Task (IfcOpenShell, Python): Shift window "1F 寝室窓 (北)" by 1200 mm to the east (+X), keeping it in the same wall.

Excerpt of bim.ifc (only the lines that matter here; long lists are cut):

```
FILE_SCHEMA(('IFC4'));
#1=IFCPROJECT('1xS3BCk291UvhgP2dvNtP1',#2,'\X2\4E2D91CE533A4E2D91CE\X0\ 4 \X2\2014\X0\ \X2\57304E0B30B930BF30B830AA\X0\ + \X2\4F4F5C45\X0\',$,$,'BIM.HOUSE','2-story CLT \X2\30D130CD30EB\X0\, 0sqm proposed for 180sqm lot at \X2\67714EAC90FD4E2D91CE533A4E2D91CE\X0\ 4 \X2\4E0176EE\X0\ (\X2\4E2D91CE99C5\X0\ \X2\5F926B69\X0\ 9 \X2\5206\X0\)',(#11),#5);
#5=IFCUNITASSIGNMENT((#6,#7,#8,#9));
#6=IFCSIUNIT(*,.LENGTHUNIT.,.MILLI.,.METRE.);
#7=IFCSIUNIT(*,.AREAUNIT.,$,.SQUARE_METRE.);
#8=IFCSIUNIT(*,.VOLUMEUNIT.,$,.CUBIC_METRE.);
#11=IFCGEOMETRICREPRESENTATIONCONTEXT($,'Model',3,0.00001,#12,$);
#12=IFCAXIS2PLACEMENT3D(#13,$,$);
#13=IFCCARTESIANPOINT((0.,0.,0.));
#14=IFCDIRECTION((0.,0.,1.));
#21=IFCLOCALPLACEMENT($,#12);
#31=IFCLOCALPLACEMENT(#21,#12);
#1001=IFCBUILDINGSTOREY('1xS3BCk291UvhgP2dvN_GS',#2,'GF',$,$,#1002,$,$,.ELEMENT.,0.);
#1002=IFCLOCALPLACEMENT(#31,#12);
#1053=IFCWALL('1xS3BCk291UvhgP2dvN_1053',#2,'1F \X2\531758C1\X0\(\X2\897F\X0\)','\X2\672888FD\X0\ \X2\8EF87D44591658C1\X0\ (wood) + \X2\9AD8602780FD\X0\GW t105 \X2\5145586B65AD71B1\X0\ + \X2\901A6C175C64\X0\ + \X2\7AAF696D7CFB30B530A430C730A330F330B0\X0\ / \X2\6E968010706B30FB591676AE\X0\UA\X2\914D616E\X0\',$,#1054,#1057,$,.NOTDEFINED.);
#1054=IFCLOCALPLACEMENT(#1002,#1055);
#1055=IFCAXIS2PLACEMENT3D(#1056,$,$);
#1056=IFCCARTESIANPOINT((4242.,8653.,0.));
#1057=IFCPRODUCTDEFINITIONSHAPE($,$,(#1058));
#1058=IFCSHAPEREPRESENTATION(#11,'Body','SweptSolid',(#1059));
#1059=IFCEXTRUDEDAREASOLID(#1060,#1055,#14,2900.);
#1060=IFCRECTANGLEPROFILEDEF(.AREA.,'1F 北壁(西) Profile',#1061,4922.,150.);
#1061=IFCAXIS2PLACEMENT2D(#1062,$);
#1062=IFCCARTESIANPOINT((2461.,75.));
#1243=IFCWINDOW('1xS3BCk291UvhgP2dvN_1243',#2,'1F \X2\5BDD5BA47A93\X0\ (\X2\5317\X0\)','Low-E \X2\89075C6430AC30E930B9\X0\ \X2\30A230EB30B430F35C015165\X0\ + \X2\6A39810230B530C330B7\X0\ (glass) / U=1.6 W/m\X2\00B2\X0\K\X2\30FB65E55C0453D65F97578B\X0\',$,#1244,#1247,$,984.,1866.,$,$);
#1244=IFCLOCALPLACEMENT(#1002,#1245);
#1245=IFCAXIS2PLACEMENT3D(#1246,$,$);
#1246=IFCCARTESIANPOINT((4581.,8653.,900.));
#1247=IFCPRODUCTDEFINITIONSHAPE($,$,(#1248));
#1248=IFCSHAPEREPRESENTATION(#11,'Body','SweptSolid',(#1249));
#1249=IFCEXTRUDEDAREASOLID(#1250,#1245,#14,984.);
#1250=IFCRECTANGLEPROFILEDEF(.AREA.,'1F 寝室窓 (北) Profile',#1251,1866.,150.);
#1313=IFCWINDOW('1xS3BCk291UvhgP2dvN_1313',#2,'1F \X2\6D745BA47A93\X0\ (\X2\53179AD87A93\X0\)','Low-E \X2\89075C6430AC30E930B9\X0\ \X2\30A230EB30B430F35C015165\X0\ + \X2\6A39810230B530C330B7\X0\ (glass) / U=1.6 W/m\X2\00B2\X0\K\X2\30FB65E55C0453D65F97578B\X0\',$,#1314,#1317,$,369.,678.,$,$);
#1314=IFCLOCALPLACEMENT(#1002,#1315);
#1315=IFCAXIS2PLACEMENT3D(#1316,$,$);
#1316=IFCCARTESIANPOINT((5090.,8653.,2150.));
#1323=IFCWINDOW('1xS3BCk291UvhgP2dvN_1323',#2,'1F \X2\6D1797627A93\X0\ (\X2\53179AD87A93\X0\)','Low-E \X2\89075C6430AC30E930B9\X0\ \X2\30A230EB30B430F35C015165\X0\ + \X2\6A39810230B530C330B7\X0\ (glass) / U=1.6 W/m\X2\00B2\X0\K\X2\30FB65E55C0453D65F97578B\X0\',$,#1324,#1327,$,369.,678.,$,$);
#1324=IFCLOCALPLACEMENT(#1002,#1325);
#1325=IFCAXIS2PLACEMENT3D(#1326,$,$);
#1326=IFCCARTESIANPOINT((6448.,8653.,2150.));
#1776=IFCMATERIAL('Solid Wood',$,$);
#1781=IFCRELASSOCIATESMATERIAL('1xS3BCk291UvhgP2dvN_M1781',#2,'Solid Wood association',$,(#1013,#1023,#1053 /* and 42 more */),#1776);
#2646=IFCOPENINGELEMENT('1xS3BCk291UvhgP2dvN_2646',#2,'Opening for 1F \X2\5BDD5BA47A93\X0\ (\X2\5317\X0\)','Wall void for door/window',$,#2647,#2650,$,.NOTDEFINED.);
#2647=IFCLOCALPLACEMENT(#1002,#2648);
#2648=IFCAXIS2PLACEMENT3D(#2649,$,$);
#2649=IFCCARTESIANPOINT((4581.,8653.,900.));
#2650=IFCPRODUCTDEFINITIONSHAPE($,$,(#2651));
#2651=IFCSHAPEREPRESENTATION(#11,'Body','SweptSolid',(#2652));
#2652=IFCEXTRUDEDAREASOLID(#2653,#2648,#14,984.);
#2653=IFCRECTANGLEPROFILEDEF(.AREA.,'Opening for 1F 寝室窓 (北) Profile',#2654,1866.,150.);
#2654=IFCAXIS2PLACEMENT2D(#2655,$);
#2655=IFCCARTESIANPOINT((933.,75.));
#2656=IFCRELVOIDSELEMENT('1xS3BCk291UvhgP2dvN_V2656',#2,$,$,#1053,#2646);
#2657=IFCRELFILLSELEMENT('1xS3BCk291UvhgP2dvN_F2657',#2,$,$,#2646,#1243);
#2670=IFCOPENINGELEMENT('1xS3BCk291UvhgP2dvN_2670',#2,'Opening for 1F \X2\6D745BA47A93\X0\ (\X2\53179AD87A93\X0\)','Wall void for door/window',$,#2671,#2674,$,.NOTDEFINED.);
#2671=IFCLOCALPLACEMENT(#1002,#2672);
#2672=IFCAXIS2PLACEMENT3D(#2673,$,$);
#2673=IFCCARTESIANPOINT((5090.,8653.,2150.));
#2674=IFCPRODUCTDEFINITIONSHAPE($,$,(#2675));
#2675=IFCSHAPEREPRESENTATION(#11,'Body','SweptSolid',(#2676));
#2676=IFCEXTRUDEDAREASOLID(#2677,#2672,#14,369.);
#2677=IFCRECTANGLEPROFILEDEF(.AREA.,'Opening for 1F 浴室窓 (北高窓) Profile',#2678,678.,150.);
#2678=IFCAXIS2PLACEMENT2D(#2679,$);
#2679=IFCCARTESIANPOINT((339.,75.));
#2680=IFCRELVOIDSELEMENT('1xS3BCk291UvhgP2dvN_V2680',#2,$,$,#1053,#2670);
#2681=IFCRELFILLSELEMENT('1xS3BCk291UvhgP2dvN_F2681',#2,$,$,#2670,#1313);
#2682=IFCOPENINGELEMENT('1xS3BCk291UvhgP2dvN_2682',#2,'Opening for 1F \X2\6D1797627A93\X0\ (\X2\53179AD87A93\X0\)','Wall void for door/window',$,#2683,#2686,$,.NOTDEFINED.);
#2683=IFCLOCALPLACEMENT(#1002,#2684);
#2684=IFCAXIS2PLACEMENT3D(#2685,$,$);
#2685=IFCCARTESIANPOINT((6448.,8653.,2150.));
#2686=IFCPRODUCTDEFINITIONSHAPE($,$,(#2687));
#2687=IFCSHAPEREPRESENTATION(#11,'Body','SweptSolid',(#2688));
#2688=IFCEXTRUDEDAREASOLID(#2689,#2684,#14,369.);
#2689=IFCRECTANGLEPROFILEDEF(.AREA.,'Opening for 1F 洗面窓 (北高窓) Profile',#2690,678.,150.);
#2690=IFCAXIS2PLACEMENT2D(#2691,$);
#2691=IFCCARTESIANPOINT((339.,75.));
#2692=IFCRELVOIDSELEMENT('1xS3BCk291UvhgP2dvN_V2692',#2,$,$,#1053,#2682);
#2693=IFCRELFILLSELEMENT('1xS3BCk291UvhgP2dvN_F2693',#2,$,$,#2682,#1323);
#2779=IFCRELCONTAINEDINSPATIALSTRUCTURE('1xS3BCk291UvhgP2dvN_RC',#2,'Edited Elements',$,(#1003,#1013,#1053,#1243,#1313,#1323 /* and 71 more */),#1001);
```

```python
import ifcopenshell
import ifcopenshell.api.geometry
import ifcopenshell.util.placement

model = ifcopenshell.open("bim.ifc")

window = model.by_guid("1xS3BCk291UvhgP2dvN_1243")
opening = window.FillsVoids[0].RelatingOpeningElement
wall = opening.VoidsElements[0].RelatingBuildingElement

wall_matrix = ifcopenshell.util.placement.get_local_placement(wall.ObjectPlacement)
shift = wall_matrix[:3, 0] * 1200.0
before = ifcopenshell.util.placement.get_local_placement(window.ObjectPlacement)[:3, 3].copy()

# The window is not placed relative to its opening, so move both.
for product in (opening, window):
    matrix = ifcopenshell.util.placement.get_local_placement(product.ObjectPlacement)
    matrix[:3, 3] += shift
    ifcopenshell.api.geometry.edit_object_placement(model, product=product, matrix=matrix, is_si=False)

after = ifcopenshell.util.placement.get_local_placement(window.ObjectPlacement)[:3, 3]
print("window moved by", (after - before).round(3) + 0.0)

model.write("bim_v2.ifc")
```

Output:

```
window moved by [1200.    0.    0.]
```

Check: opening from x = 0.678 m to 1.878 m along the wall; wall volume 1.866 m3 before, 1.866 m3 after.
